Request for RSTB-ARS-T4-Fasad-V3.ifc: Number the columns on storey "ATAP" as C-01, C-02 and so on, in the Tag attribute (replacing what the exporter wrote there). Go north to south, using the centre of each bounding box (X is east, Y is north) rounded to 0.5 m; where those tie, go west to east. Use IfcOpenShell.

First a look at what the model holds.

```python
import ifcopenshell
import ifcopenshell.util.element
import ifcopenshell.util.placement

model = ifcopenshell.open("RSTB-ARS-T4-Fasad-V3.ifc")
print(model.schema)
storey = next(s for s in model.by_type("IfcBuildingStorey") if s.Name == "ATAP")
columns = [e for e in ifcopenshell.util.element.get_decomposition(storey) if e.is_a("IfcColumn")]
for e in sorted(columns, key=lambda e: e.id()):
    origin = ifcopenshell.util.placement.get_local_placement(e.ObjectPlacement)[:3, 3]
    print(e.id(), e.Tag, e.Name, origin.round(2) + 0.0, sep=" | ")
```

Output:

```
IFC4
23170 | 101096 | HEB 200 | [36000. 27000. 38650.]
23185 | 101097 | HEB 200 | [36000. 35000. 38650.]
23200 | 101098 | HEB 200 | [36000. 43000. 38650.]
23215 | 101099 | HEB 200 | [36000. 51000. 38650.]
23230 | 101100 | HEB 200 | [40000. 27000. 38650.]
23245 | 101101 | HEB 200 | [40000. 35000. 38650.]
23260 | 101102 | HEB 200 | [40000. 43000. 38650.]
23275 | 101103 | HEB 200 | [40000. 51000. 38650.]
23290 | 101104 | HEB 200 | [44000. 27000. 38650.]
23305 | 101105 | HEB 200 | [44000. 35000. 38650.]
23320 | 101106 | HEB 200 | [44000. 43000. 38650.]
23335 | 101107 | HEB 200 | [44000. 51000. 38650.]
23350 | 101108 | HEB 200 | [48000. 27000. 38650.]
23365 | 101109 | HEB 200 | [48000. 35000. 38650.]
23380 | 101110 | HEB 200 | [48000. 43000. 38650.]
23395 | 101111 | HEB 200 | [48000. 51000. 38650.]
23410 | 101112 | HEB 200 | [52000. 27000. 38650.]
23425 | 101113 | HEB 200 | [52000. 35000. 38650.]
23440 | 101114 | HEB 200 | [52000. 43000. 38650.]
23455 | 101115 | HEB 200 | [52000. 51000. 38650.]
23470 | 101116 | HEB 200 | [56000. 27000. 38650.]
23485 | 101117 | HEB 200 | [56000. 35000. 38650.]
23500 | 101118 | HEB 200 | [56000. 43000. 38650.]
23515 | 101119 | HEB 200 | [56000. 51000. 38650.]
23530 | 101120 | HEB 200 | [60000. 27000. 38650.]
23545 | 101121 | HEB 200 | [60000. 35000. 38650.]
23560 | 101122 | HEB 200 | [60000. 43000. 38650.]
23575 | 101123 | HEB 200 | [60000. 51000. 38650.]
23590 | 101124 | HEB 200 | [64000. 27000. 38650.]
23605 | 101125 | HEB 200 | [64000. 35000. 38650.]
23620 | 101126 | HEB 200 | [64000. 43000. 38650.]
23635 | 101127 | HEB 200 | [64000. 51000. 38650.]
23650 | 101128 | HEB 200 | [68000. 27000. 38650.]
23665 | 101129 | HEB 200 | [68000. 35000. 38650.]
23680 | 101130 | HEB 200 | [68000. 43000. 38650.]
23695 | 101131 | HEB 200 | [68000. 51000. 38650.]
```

```python
import ifcopenshell
import ifcopenshell.geom
import ifcopenshell.util.element
import ifcopenshell.util.shape

model = ifcopenshell.open("RSTB-ARS-T4-Fasad-V3.ifc")
settings = ifcopenshell.geom.settings()
settings.set("use-world-coords", True)


def centre(element):
    shape = ifcopenshell.geom.create_shape(settings, element)
    return ifcopenshell.util.shape.get_bbox_centroid(shape.geometry)


storey = next(s for s in model.by_type("IfcBuildingStorey") if s.Name == "ATAP")
columns = [e for e in ifcopenshell.util.element.get_decomposition(storey) if e.is_a("IfcColumn")]

# Insertion points can sit at a corner or the storey origin, so sort by the geometry (in metres).
centres = {e: centre(e) for e in columns}
columns.sort(key=lambda e: (-round(centres[e][1] / 0.5), centres[e][0]))

for i, e in enumerate(columns, start=1):
    number = f"C-{i:02d}"
    e.Tag = number
    print(e.id(), number)

model.write("RSTB-ARS-T4-Fasad-V3_v2.ifc")
```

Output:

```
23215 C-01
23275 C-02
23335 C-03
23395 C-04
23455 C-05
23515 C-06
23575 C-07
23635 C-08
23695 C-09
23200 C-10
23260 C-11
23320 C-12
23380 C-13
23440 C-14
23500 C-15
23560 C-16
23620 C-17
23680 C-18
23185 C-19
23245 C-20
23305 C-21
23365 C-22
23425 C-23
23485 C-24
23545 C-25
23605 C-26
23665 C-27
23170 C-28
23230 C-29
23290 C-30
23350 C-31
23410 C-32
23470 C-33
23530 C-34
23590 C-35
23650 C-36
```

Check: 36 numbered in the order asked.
